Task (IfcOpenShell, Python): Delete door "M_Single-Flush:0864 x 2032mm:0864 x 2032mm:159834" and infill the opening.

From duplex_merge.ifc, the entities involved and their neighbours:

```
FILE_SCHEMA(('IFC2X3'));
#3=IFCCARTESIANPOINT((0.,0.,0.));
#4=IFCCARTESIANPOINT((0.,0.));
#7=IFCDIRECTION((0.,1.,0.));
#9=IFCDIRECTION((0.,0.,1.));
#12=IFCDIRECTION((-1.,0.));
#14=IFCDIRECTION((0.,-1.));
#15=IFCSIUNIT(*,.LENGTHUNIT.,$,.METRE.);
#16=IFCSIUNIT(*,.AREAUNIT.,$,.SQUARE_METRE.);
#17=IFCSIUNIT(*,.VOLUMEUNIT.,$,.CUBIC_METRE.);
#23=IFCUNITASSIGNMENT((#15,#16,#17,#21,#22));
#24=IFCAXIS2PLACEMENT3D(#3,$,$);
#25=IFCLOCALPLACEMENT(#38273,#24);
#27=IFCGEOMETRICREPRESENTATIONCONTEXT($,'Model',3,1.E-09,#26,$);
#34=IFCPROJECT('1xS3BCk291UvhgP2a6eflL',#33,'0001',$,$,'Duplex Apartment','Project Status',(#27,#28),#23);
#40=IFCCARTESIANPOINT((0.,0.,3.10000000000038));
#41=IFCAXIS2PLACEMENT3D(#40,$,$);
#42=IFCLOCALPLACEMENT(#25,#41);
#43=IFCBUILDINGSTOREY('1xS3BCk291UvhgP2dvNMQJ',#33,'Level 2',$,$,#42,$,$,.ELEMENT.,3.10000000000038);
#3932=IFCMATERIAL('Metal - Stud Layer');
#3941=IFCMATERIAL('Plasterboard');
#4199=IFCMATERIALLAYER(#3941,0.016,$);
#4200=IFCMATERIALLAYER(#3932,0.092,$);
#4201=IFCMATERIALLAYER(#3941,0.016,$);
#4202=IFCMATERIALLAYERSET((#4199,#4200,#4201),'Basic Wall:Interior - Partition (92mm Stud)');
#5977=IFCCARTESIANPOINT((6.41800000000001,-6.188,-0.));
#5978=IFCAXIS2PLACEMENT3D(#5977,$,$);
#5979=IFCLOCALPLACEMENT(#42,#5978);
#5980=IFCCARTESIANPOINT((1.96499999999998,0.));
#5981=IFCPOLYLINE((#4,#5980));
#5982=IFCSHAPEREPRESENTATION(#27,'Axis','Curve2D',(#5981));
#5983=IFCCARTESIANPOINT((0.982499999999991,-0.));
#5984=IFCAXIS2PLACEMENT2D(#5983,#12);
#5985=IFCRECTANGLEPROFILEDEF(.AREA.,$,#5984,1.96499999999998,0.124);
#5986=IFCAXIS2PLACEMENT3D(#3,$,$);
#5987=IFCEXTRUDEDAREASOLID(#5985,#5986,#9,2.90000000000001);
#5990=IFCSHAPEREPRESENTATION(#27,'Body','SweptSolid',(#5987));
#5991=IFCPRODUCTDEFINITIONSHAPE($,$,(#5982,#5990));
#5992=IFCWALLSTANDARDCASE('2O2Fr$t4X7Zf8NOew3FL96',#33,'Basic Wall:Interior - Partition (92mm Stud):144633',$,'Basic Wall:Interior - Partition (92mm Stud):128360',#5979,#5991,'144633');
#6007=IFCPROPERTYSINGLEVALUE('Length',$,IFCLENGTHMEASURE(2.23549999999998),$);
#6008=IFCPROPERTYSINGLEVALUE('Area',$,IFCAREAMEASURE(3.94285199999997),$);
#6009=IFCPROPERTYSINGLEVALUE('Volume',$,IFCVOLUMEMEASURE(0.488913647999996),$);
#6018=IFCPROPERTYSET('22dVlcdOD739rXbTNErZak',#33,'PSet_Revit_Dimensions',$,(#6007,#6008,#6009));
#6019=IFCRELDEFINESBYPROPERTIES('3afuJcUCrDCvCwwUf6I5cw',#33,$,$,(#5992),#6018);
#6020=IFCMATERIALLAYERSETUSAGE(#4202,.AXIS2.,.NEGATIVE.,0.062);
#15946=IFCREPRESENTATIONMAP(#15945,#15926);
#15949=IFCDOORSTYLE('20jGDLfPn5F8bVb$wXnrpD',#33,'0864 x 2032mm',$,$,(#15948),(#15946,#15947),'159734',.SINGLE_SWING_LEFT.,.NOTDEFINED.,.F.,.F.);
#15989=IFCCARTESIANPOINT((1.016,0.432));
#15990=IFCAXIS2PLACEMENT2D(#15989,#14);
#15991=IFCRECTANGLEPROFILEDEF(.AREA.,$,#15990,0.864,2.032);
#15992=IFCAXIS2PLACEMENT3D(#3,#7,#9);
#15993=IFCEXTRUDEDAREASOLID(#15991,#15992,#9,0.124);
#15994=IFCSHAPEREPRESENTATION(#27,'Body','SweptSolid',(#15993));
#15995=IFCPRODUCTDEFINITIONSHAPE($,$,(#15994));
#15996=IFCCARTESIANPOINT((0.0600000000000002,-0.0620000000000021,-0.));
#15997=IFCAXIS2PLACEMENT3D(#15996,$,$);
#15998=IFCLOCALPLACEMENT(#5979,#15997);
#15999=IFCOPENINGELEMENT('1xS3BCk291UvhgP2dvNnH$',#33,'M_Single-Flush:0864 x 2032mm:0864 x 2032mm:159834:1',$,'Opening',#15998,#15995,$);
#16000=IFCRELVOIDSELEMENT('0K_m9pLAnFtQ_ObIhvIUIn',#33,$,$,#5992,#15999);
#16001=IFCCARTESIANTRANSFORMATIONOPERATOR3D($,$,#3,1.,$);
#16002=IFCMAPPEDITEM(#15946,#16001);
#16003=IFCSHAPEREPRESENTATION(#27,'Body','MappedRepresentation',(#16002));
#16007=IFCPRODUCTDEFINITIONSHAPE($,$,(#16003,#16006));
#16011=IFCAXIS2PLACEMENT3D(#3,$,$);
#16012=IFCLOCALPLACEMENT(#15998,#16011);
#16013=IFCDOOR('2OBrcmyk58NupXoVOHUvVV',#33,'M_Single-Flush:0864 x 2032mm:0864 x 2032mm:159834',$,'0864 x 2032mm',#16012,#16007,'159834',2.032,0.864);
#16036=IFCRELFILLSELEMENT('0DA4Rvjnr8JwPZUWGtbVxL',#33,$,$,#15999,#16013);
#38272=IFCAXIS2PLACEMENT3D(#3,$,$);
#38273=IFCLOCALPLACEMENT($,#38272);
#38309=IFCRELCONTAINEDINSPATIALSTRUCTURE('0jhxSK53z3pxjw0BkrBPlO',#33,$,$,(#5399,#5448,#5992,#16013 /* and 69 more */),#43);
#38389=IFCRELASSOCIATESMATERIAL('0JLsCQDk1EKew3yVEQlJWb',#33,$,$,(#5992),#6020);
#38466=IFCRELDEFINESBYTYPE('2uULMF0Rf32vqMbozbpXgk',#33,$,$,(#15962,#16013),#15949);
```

```python
import ifcopenshell
import ifcopenshell.api.feature
import ifcopenshell.api.pset
import ifcopenshell.api.root
import ifcopenshell.geom
import ifcopenshell.util.element
import ifcopenshell.util.shape
import ifcopenshell.util.unit

model = ifcopenshell.open("duplex_merge.ifc")
area_scale = ifcopenshell.util.unit.calculate_unit_scale(model, "AREAUNIT")
volume_scale = ifcopenshell.util.unit.calculate_unit_scale(model, "VOLUMEUNIT")
settings = ifcopenshell.geom.settings()


def volume(element):
    """Net volume in cubic metres, openings subtracted."""
    shape = ifcopenshell.geom.create_shape(settings, element)
    return ifcopenshell.util.shape.get_volume(shape.geometry)


door = model.by_guid("2OBrcmyk58NupXoVOHUvVV")
opening = door.FillsVoids[0].RelatingOpeningElement
wall = opening.VoidsElements[0].RelatingBuildingElement
before = volume(wall)

ifcopenshell.api.root.remove_product(model, product=door)
ifcopenshell.api.feature.remove_feature(model, feature=opening)

after = volume(wall)
thickness = 0.124  # wall thickness in metres

# Update the wall's stored quantities.
pset = model.by_id(ifcopenshell.util.element.get_pset(wall, "PSet_Revit_Dimensions", should_inherit=False)["id"])
ifcopenshell.api.pset.edit_pset(model, pset=pset, properties={
    "Area": model.create_entity("IfcAreaMeasure", after / thickness / area_scale),
    "Volume": model.create_entity("IfcVolumeMeasure", after / volume_scale),
})

print(f"wall volume {before:.3f} -> {after:.3f} m3")

model.write("duplex_merge-out.ifc")
```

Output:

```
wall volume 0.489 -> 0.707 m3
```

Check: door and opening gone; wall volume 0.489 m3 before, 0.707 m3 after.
